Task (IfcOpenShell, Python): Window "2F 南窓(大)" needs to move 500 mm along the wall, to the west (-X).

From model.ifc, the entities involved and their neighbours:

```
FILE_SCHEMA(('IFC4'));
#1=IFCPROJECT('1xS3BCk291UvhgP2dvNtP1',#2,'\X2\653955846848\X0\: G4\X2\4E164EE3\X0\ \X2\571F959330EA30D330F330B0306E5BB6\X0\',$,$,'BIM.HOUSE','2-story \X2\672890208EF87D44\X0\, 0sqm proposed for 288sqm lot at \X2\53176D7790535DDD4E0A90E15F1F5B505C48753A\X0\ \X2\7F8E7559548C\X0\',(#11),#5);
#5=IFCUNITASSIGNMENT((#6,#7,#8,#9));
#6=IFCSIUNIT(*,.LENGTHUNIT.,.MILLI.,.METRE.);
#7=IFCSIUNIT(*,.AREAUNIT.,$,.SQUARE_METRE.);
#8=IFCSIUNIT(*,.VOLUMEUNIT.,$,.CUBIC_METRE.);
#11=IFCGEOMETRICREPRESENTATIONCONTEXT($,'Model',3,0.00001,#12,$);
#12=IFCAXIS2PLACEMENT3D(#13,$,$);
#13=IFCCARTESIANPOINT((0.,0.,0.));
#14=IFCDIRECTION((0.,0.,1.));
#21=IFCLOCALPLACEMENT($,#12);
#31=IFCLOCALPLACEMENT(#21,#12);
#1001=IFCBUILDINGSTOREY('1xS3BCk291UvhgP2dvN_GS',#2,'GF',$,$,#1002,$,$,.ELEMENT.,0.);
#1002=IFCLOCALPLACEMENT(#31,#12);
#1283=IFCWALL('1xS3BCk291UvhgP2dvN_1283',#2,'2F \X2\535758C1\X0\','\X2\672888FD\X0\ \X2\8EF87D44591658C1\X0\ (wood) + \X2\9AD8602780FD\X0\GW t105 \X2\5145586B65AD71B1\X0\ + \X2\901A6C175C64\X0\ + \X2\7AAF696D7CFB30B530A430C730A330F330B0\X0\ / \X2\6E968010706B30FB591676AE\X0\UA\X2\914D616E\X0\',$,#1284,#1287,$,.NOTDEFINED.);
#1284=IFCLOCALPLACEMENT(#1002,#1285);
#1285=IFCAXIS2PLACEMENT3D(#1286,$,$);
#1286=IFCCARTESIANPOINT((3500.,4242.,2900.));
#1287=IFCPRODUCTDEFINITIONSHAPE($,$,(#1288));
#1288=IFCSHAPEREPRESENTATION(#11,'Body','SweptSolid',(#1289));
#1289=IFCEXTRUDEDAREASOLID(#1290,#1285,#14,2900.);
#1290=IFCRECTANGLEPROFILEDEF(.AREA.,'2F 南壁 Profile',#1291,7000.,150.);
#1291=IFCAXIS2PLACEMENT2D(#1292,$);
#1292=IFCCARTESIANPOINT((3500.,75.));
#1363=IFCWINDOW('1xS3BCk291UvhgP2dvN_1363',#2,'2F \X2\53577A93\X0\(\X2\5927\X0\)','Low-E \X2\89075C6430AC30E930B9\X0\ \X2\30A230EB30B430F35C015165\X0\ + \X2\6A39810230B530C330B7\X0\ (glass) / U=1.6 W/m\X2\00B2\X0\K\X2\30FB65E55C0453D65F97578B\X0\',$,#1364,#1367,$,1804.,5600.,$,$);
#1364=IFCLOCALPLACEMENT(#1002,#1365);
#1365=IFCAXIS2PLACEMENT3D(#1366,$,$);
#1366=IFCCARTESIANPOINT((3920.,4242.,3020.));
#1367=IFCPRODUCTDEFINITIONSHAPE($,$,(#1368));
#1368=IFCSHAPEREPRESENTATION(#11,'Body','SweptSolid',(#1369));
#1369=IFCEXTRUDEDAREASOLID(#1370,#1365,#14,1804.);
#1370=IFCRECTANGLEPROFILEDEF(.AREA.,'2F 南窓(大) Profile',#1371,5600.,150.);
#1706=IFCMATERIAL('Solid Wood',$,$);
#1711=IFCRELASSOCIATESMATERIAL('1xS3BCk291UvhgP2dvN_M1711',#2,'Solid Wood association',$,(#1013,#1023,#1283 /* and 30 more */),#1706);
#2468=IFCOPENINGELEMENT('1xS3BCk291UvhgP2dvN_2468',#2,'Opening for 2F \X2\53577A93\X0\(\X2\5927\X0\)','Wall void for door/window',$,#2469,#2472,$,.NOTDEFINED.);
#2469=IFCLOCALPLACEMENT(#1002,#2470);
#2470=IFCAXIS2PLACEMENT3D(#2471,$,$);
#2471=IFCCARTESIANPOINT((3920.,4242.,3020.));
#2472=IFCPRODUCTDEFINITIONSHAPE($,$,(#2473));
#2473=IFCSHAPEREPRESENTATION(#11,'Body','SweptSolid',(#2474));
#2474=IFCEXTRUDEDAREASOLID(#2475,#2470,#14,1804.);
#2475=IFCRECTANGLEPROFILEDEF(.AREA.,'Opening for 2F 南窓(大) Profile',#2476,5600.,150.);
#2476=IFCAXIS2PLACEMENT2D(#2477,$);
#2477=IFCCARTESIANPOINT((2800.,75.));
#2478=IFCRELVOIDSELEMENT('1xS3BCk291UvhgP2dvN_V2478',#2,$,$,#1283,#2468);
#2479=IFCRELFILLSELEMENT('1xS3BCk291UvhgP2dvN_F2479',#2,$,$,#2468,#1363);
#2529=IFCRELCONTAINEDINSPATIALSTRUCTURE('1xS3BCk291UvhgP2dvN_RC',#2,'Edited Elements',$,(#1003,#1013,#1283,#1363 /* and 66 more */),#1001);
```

```python
import ifcopenshell
import ifcopenshell.api.geometry
import ifcopenshell.util.placement

model = ifcopenshell.open("model.ifc")

window = model.by_guid("1xS3BCk291UvhgP2dvN_1363")
opening = window.FillsVoids[0].RelatingOpeningElement
wall = opening.VoidsElements[0].RelatingBuildingElement

wall_matrix = ifcopenshell.util.placement.get_local_placement(wall.ObjectPlacement)
shift = wall_matrix[:3, 0] * -500.0
before = ifcopenshell.util.placement.get_local_placement(window.ObjectPlacement)[:3, 3].copy()

# The window is not placed relative to its opening, so move both.
for product in (opening, window):
    matrix = ifcopenshell.util.placement.get_local_placement(product.ObjectPlacement)
    matrix[:3, 3] += shift
    ifcopenshell.api.geometry.edit_object_placement(model, product=product, matrix=matrix, is_si=False)

after = ifcopenshell.util.placement.get_local_placement(window.ObjectPlacement)[:3, 3]
print("window moved by", (after - before).round(3) + 0.0)

model.write("model_rev.ifc")
```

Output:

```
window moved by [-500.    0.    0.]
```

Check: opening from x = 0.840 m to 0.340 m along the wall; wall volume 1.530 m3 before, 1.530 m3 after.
